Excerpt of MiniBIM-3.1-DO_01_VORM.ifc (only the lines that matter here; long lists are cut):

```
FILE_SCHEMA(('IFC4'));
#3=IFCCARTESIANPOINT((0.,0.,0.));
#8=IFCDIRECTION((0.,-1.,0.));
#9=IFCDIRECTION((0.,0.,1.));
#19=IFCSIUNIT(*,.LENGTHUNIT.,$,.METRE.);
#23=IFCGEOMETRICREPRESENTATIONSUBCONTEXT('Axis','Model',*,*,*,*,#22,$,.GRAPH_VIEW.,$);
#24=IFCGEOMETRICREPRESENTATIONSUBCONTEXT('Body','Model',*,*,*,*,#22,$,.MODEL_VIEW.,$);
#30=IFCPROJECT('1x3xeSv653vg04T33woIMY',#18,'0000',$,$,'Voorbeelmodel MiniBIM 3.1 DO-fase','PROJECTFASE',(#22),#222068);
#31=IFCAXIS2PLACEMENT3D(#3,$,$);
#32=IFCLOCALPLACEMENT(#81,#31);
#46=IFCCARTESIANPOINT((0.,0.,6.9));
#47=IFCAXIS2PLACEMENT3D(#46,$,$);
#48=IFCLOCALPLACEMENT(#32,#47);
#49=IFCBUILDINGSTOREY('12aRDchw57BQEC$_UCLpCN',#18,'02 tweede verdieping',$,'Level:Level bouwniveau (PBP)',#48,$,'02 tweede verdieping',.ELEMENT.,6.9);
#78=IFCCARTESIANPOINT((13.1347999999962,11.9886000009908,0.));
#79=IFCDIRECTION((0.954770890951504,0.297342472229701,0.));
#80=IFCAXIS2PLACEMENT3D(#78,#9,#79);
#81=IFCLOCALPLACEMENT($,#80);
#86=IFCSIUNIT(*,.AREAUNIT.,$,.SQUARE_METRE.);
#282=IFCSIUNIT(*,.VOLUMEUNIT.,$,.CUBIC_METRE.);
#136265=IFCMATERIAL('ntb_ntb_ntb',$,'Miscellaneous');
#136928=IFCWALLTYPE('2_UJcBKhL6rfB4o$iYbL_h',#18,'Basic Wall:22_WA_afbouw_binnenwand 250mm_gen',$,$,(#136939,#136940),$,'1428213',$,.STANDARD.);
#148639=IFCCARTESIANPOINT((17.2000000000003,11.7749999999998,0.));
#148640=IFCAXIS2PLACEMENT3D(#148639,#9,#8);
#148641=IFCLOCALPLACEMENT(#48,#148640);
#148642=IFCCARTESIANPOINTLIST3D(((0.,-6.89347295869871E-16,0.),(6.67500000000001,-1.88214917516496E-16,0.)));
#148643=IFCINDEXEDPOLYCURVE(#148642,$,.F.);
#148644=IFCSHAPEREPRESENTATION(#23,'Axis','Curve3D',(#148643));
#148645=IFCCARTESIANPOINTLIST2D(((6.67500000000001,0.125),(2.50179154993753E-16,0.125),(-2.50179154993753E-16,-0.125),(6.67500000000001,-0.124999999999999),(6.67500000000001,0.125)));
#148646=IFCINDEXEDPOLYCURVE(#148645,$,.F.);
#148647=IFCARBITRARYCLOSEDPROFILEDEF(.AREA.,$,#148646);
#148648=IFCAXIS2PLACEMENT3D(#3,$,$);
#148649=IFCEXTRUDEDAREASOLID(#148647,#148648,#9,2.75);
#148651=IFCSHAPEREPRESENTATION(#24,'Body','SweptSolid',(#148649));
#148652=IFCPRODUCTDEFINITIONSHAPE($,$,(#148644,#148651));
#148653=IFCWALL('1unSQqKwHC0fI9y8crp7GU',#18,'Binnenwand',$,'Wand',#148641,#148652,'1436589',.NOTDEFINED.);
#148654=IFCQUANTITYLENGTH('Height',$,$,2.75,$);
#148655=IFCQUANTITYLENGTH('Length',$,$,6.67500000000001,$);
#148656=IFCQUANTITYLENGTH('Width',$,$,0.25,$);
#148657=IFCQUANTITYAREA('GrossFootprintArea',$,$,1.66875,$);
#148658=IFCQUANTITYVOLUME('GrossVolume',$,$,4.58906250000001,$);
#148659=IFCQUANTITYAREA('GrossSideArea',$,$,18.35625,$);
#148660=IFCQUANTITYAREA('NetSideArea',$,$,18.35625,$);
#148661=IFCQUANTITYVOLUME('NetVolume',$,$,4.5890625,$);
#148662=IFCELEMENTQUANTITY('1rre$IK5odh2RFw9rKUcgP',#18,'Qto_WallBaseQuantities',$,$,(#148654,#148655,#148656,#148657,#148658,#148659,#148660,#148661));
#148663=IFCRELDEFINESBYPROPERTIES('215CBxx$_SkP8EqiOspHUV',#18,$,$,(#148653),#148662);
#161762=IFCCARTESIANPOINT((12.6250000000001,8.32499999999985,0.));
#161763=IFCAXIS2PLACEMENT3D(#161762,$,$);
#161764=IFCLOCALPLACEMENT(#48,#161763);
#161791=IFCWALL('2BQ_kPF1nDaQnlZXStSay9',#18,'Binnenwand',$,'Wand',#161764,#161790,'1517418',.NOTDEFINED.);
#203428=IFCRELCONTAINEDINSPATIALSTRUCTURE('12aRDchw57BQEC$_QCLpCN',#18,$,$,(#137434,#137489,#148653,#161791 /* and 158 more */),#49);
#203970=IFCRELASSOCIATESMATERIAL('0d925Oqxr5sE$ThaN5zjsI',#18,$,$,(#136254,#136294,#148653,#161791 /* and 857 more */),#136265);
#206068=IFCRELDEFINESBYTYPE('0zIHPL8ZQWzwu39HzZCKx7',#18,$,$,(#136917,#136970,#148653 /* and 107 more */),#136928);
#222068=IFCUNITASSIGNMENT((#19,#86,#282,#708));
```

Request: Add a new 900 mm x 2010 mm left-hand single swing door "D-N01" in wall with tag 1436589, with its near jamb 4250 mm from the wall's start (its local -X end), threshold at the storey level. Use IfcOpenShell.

```python
import numpy as np
import ifcopenshell
import ifcopenshell.api.feature
import ifcopenshell.api.geometry
import ifcopenshell.api.pset
import ifcopenshell.api.root
import ifcopenshell.api.spatial
import ifcopenshell.geom
import ifcopenshell.util.element
import ifcopenshell.util.placement
import ifcopenshell.util.representation
import ifcopenshell.util.shape
import ifcopenshell.util.unit

model = ifcopenshell.open("MiniBIM-3.1-DO_01_VORM.ifc")
unit_scale = ifcopenshell.util.unit.calculate_unit_scale(model)
area_scale = ifcopenshell.util.unit.calculate_unit_scale(model, "AREAUNIT")
volume_scale = ifcopenshell.util.unit.calculate_unit_scale(model, "VOLUMEUNIT")
settings = ifcopenshell.geom.settings()


def volume(element):
    """Net volume in cubic metres, openings subtracted."""
    shape = ifcopenshell.geom.create_shape(settings, element)
    return ifcopenshell.util.shape.get_volume(shape.geometry)


wall = model.by_guid("1unSQqKwHC0fI9y8crp7GU")
storey = ifcopenshell.util.element.get_container(wall, ifc_class="IfcBuildingStorey")
context = ifcopenshell.util.representation.get_context(model, "Model", "Body", "MODEL_VIEW")
before = volume(wall)

width, height, from_end, sill = 0.9, 2.01, 4.25, 0.0  # metres

# The wall runs along its own X axis, and the end named is its -X end.
wall_shape = ifcopenshell.geom.create_shape(settings, wall)
x, y, z = ifcopenshell.util.shape.get_vertices(wall_shape.geometry).T
start = x.min() + from_end
face, thickness = float(y.min()), float(y.max() - y.min())
wall_matrix = ifcopenshell.util.placement.get_local_placement(wall.ObjectPlacement)
level = ifcopenshell.util.placement.get_local_placement(storey.ObjectPlacement)[2, 3]


def in_wall(x, y):
    """Placement at x, y metres in the wall's axes, at sill height."""
    matrix = wall_matrix.copy()
    matrix[:, 3] = wall_matrix @ np.array([x / unit_scale, y / unit_scale, 0.0, 1.0])
    matrix[2, 3] = level + sill / unit_scale
    return matrix


# Opening: a box that overshoots both wall faces by 50 mm.
opening = ifcopenshell.api.root.create_entity(model, ifc_class="IfcOpeningElement", predefined_type="OPENING")
box = ifcopenshell.api.geometry.add_wall_representation(
    model, context=context, length=width, height=height, thickness=thickness + 0.1
)
ifcopenshell.api.geometry.assign_representation(model, product=opening, representation=box)
ifcopenshell.api.geometry.edit_object_placement(model, product=opening, matrix=in_wall(start, face - 0.05), is_si=False)
ifcopenshell.api.feature.add_feature(model, feature=opening, element=wall)

door = ifcopenshell.api.root.create_entity(model, ifc_class="IfcDoor", name="D-N01", predefined_type="DOOR")
door.OverallWidth, door.OverallHeight = width / unit_scale, height / unit_scale
door.OperationType = "SINGLE_SWING_LEFT"
body = ifcopenshell.api.geometry.add_door_representation(
    model,
    context=context,
    overall_width=door.OverallWidth,
    overall_height=door.OverallHeight,
    operation_type="SINGLE_SWING_LEFT",
    lining_properties={"LiningDepth": thickness / unit_scale, "ThresholdDepth": thickness / unit_scale},
)
ifcopenshell.api.geometry.assign_representation(model, product=door, representation=body)
ifcopenshell.api.spatial.assign_container(model, products=[door], relating_structure=storey)
ifcopenshell.api.feature.add_filling(model, opening=opening, element=door)

# The lining spans the wall, so the door starts at the wall face.
ifcopenshell.api.geometry.edit_object_placement(model, product=door, matrix=in_wall(start, face), is_si=False)

after = volume(wall)

# Update the wall's stored quantities.
qto = model.by_id(ifcopenshell.util.element.get_pset(wall, "Qto_WallBaseQuantities", should_inherit=False)["id"])
ifcopenshell.api.pset.edit_qto(model, qto=qto, properties={
    "NetSideArea": after / thickness / area_scale,
    "NetVolume": after / volume_scale,
})

print(f"wall volume {before:.3f} -> {after:.3f} m3")

model.write("MiniBIM-3.1-DO_01_VORM_updated.ifc")
```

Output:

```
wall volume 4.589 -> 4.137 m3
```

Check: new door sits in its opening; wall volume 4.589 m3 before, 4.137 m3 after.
